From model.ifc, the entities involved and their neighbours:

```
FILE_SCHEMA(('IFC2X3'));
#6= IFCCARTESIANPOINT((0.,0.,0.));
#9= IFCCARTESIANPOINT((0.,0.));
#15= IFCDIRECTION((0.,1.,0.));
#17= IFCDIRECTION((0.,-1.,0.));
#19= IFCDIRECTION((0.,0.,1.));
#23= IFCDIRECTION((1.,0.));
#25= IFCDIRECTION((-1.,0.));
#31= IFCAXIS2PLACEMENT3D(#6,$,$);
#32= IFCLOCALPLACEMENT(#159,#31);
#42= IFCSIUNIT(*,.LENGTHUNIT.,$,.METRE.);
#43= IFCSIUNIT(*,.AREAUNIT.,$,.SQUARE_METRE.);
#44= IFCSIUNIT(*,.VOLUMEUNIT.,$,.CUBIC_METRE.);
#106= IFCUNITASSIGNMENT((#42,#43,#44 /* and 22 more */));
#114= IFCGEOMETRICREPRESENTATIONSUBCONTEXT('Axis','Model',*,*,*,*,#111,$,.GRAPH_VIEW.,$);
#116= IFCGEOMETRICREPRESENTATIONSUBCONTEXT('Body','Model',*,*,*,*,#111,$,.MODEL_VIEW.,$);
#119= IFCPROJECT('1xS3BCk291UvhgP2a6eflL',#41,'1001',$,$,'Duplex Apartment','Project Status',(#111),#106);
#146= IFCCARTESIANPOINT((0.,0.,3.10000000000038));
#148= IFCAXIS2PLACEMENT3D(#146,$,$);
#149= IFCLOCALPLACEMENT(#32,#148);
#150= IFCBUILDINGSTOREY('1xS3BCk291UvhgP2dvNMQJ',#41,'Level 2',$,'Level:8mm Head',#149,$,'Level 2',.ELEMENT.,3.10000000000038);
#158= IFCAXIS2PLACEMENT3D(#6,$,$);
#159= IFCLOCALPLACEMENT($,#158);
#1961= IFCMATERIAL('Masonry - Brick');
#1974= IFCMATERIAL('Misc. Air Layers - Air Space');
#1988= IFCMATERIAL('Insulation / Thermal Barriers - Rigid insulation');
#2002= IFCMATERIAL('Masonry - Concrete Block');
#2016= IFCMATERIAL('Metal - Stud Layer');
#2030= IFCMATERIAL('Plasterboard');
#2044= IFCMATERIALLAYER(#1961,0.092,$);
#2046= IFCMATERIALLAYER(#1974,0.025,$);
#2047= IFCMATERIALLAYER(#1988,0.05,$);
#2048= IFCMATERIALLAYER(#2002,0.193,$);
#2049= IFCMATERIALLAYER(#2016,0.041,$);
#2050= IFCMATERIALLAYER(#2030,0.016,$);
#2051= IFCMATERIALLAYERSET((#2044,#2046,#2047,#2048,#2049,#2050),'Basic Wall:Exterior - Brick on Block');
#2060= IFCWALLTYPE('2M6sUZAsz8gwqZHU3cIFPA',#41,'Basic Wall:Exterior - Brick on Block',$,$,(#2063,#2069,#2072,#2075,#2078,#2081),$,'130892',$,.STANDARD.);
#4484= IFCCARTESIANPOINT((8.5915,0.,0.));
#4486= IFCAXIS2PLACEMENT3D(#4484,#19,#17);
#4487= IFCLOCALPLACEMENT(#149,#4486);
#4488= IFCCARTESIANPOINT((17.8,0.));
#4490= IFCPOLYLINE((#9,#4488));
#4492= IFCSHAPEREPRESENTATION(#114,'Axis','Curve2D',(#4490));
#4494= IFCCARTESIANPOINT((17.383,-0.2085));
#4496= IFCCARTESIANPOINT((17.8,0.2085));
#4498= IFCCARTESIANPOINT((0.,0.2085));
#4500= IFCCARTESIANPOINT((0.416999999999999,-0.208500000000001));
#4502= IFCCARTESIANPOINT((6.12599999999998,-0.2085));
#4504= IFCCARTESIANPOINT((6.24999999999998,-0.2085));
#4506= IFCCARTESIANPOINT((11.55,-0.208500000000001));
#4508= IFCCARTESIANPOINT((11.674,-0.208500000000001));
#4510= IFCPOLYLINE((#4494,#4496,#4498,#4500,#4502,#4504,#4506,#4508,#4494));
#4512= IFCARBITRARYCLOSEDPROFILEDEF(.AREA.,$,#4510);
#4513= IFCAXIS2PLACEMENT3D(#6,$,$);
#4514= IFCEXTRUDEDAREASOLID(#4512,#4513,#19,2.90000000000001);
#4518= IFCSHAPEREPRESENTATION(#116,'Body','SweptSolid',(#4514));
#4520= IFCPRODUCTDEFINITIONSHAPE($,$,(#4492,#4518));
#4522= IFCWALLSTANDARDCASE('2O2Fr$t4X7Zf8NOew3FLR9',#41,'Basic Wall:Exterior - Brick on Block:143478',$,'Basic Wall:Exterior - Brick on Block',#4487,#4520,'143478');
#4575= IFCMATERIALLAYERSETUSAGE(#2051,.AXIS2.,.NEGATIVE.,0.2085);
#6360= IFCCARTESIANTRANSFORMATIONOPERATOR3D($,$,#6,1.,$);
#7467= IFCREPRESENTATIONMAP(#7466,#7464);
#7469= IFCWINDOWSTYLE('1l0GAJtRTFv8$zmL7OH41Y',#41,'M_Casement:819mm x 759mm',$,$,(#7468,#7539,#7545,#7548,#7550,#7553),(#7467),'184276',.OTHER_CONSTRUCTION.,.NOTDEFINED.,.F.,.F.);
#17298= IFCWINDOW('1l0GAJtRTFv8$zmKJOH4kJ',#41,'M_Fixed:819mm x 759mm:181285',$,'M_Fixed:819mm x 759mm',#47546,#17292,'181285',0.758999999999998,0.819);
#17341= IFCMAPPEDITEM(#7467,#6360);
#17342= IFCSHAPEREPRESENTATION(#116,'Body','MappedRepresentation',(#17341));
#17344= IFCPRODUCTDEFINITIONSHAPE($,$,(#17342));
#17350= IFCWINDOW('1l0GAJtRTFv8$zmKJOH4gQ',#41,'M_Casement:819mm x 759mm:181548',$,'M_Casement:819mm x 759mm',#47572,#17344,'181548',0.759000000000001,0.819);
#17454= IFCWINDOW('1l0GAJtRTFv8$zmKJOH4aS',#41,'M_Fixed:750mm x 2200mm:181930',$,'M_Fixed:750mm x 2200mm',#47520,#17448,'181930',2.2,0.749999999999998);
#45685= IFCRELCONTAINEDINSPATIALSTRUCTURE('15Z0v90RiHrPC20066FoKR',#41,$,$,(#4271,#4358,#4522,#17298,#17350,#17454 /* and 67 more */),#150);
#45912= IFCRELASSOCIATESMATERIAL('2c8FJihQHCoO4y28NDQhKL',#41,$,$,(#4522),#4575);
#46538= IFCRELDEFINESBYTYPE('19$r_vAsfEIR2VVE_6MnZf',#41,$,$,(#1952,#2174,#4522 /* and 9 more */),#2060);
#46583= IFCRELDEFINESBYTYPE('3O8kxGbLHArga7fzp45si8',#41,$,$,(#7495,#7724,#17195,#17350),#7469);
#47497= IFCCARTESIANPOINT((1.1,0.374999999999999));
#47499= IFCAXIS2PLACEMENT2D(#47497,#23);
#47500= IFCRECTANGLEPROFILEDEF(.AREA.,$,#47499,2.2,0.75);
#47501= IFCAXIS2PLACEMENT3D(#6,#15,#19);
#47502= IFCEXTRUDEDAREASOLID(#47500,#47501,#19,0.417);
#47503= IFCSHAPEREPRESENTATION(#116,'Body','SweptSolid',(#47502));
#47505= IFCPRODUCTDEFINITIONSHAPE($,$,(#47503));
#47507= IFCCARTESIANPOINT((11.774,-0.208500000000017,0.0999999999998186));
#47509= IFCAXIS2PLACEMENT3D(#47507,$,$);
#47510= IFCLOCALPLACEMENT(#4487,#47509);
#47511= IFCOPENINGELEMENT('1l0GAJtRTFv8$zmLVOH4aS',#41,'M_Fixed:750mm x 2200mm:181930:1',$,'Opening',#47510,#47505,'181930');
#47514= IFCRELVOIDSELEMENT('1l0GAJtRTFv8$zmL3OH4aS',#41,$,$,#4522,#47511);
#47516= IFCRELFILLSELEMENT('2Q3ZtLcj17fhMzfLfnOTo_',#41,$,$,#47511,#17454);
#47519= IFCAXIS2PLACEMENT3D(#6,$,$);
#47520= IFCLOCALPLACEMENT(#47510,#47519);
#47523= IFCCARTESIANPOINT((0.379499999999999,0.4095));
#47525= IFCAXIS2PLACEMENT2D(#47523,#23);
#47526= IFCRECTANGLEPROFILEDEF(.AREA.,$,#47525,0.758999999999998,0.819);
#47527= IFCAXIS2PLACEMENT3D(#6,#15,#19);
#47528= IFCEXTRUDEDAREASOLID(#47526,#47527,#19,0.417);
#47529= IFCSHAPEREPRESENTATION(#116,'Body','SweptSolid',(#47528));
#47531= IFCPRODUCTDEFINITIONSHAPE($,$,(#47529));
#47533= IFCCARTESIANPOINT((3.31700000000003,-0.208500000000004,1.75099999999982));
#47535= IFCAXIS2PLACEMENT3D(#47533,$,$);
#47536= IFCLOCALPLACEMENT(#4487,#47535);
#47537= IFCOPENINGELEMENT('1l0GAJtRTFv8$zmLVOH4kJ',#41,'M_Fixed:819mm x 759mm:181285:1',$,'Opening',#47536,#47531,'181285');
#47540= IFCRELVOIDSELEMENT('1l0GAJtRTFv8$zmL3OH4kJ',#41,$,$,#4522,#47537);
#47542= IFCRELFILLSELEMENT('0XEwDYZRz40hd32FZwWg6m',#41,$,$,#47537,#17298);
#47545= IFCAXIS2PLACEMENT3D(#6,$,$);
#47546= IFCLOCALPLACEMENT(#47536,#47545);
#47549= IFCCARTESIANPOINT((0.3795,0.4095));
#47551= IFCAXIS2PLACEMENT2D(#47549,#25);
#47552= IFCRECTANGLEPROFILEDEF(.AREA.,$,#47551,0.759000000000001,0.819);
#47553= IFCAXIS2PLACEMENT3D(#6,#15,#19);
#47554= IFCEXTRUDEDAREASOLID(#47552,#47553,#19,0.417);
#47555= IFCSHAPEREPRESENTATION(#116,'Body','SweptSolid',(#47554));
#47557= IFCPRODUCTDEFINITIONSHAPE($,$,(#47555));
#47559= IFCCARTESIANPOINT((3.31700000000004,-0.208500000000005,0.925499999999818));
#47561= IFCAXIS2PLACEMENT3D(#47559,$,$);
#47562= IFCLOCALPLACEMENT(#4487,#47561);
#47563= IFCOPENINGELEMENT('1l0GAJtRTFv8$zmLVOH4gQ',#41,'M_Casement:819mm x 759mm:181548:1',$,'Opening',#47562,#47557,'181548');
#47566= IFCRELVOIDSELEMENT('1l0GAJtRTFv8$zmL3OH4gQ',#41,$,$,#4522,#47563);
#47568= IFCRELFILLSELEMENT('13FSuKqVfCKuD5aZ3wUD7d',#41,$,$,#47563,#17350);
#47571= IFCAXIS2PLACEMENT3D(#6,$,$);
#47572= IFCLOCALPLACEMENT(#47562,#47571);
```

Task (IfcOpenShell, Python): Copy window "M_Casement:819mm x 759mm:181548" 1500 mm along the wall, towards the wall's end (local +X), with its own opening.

```python
import ifcopenshell
import ifcopenshell.api.feature
import ifcopenshell.api.geometry
import ifcopenshell.api.root
import ifcopenshell.geom
import ifcopenshell.util.element
import ifcopenshell.util.placement
import ifcopenshell.util.shape
import ifcopenshell.util.unit

model = ifcopenshell.open("model.ifc")
unit_scale = ifcopenshell.util.unit.calculate_unit_scale(model)
settings = ifcopenshell.geom.settings()


def volume(element):
    """Net volume in cubic metres, openings subtracted."""
    shape = ifcopenshell.geom.create_shape(settings, element)
    return ifcopenshell.util.shape.get_volume(shape.geometry)


def reuse_history(source, copy):
    """copy_class also copies each property set's owner history, people and application; keep the originals."""
    for rel in copy.IsDefinedBy:
        if rel.is_a("IfcRelDefinesByProperties") and (history := rel.RelatingPropertyDefinition.OwnerHistory):
            rel.RelatingPropertyDefinition.OwnerHistory = source.OwnerHistory
            ifcopenshell.util.element.remove_deep2(model, history)


window = model.by_guid("1l0GAJtRTFv8$zmKJOH4gQ")
opening = window.FillsVoids[0].RelatingOpeningElement
wall = opening.VoidsElements[0].RelatingBuildingElement
before = volume(wall)
shift = ifcopenshell.util.placement.get_local_placement(wall.ObjectPlacement)[:3, 0] * 1.5 / unit_scale

# copy_class copies the void relationship, type, container and properties, but no geometry.
new_opening = ifcopenshell.api.root.copy_class(model, product=opening)
new_opening.Representation = ifcopenshell.util.element.copy_deep(
    model, opening.Representation, exclude=["IfcGeometricRepresentationContext", "IfcRepresentationMap"]
)
new_opening.Name = "M_Casement:819mm x 759mm"
new_opening.Tag = None
new_window = ifcopenshell.api.root.copy_class(model, product=window)
new_window.Representation = ifcopenshell.util.element.copy_deep(
    model, window.Representation, exclude=["IfcGeometricRepresentationContext", "IfcRepresentationMap"]
)
new_window.Name = "M_Casement:819mm x 759mm"
new_window.Tag = None
reuse_history(window, new_window)
fills = ifcopenshell.api.feature.add_filling(model, opening=new_opening, element=new_window)
fills.OwnerHistory = new_window.OwnerHistory  # required in IFC2X3

for old, new in ((opening, new_opening), (window, new_window)):
    matrix = ifcopenshell.util.placement.get_local_placement(old.ObjectPlacement)
    matrix[:3, 3] += shift
    ifcopenshell.api.geometry.edit_object_placement(model, product=new, matrix=matrix, is_si=False)

after = volume(wall)

print(f"wall volume {before:.3f} -> {after:.3f} m3")

model.write("model_edited.ifc")
```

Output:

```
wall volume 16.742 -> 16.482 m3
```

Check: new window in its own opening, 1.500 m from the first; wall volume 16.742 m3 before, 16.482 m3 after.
